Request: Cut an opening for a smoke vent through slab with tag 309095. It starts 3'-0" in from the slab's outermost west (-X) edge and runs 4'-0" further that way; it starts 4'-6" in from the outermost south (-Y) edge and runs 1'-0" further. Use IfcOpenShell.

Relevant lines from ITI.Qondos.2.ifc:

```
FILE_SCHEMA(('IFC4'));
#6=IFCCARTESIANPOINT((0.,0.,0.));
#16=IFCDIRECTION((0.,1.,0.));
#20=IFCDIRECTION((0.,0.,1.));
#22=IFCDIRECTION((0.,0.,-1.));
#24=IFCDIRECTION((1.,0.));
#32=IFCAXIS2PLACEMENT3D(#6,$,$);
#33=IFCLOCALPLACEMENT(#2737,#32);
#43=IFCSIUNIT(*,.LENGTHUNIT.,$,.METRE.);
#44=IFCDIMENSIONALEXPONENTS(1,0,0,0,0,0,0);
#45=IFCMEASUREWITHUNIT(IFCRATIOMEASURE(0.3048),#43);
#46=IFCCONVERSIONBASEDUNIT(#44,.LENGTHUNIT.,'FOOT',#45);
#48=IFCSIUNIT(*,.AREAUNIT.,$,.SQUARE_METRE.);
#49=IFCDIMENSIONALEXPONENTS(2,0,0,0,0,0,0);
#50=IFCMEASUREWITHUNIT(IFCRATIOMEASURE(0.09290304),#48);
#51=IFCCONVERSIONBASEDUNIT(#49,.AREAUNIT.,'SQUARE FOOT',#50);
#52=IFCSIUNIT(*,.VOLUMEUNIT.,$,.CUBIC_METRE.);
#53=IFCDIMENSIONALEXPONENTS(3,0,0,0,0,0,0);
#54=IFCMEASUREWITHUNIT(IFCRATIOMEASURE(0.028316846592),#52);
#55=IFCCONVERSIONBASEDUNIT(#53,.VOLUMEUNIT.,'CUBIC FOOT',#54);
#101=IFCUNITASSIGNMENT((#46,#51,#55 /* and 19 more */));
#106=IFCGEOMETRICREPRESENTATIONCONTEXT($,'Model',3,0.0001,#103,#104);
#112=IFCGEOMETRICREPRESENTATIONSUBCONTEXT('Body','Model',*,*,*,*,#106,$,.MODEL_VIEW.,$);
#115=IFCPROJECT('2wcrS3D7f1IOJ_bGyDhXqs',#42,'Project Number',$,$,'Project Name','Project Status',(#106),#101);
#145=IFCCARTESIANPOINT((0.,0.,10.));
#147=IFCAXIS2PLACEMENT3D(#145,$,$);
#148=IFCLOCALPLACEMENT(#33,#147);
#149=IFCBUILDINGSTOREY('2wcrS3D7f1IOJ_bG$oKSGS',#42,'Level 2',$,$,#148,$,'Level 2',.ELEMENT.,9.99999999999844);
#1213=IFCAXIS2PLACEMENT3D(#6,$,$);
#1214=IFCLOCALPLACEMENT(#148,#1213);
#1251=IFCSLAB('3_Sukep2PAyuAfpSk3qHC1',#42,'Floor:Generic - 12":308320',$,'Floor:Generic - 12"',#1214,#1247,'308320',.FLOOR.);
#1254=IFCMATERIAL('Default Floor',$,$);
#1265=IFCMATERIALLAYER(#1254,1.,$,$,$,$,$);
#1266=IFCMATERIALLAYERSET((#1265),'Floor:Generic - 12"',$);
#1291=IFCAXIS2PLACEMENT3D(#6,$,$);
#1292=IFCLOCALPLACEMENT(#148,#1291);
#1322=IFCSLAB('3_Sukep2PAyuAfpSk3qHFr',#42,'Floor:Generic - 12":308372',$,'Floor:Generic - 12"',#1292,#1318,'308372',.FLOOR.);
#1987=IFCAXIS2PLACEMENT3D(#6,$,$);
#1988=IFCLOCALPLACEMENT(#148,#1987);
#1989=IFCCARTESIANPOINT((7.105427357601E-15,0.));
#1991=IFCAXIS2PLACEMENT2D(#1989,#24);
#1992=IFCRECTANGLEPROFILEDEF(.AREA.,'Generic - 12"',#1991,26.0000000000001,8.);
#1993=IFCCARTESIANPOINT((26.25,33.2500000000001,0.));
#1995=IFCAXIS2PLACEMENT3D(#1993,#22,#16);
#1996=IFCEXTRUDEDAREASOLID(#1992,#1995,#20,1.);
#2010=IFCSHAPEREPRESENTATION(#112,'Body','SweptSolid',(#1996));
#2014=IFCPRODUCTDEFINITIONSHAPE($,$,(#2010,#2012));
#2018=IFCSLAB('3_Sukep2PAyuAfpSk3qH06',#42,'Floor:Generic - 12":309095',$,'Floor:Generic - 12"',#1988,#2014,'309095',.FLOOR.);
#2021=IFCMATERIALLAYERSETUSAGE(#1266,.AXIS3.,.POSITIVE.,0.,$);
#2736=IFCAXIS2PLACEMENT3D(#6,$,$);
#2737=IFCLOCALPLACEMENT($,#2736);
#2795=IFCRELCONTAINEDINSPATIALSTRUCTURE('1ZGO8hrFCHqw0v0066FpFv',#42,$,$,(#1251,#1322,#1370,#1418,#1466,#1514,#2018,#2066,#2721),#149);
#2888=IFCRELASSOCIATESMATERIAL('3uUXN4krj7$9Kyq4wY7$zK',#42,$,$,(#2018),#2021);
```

```python
import numpy as np
import ifcopenshell
import ifcopenshell.api.feature
import ifcopenshell.api.geometry
import ifcopenshell.api.root
import ifcopenshell.geom
import ifcopenshell.util.placement
import ifcopenshell.util.representation
import ifcopenshell.util.shape
import ifcopenshell.util.unit

model = ifcopenshell.open("ITI.Qondos.2.ifc")
unit_scale = ifcopenshell.util.unit.calculate_unit_scale(model)
settings = ifcopenshell.geom.settings()


def volume(element):
    """Net volume in cubic metres, openings subtracted."""
    shape = ifcopenshell.geom.create_shape(settings, element)
    return ifcopenshell.util.shape.get_volume(shape.geometry)


slab = model.by_guid("3_Sukep2PAyuAfpSk3qH06")
before = volume(slab)

# Extent in the slab's own axes, in metres. The edges named are its -X and -Y sides.
slab_shape = ifcopenshell.geom.create_shape(settings, slab)
vertices = ifcopenshell.util.shape.get_vertices(slab_shape.geometry)
x_min, y_min, bottom = vertices.min(axis=0)
top = vertices[:, 2].max()

opening = ifcopenshell.api.root.create_entity(model, ifc_class="IfcOpeningElement", name="Smoke vent opening", predefined_type="OPENING")
context = ifcopenshell.util.representation.get_context(model, "Model", "Body", "MODEL_VIEW")
width, depth = 1.2192, 0.3048
outline = [(0.0, 0.0), (width, 0.0), (width, depth), (0.0, depth), (0.0, 0.0)]
# Overshoot both faces by 50 mm so the cut is clean.
shape = ifcopenshell.api.geometry.add_slab_representation(
    model, context=context, depth=top - bottom + 0.1, polyline=outline
)
ifcopenshell.api.geometry.assign_representation(model, product=opening, representation=shape)

matrix = ifcopenshell.util.placement.get_local_placement(slab.ObjectPlacement)
matrix[:, 3] = matrix @ np.append(np.array([x_min + 0.9144, y_min + 1.3716, bottom - 0.05]) / unit_scale, 1.0)
ifcopenshell.api.geometry.edit_object_placement(model, product=opening, matrix=matrix, is_si=False)
ifcopenshell.api.feature.add_feature(model, feature=opening, element=slab)

after = volume(slab)

print(f"slab volume {before:.3f} -> {after:.3f} m3")

model.write("ITI.Qondos.2_updated.ifc")
```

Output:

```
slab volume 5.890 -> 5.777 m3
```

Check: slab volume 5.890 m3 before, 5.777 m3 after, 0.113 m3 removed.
